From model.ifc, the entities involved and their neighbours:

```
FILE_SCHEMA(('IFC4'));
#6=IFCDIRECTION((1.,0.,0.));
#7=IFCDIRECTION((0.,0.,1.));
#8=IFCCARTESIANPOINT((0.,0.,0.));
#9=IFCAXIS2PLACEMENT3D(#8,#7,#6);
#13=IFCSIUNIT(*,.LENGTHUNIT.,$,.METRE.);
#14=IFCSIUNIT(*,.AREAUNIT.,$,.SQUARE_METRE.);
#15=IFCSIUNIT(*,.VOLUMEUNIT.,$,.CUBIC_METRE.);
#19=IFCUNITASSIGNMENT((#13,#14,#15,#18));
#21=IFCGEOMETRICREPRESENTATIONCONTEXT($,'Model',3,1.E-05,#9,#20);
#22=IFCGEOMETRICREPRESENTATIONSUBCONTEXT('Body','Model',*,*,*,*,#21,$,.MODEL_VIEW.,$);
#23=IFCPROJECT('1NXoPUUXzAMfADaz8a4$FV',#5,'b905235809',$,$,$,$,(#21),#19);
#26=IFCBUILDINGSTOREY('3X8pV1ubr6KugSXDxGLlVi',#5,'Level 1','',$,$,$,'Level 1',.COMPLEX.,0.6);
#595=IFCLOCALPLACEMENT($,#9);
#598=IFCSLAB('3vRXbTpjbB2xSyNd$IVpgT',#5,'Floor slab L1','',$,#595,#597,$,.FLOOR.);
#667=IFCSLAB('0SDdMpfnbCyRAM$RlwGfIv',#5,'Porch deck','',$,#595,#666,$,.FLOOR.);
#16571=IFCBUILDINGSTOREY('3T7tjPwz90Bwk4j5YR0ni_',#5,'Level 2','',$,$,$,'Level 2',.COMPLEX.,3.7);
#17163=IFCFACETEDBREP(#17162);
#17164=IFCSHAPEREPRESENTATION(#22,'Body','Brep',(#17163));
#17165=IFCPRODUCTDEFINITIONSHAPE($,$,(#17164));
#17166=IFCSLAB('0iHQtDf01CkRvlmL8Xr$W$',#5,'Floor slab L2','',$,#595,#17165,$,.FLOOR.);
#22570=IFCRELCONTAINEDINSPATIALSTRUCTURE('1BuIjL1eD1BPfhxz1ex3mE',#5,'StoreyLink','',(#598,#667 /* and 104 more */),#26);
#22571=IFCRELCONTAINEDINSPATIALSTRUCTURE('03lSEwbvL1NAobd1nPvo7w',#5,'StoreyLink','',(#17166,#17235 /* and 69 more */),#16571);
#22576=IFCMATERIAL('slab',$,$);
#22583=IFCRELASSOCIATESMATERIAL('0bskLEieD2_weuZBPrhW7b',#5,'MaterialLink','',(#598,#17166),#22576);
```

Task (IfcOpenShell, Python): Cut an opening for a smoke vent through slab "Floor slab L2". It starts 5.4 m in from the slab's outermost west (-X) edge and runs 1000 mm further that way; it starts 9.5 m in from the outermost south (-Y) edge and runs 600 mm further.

```python
import numpy as np
import ifcopenshell
import ifcopenshell.api.feature
import ifcopenshell.api.geometry
import ifcopenshell.api.root
import ifcopenshell.geom
import ifcopenshell.util.placement
import ifcopenshell.util.representation
import ifcopenshell.util.shape
import ifcopenshell.util.unit

model = ifcopenshell.open("model.ifc")
unit_scale = ifcopenshell.util.unit.calculate_unit_scale(model)
settings = ifcopenshell.geom.settings()


def volume(element):
    """Net volume in cubic metres, openings subtracted."""
    shape = ifcopenshell.geom.create_shape(settings, element)
    return ifcopenshell.util.shape.get_volume(shape.geometry)


slab = model.by_guid("0iHQtDf01CkRvlmL8Xr$W$")
before = volume(slab)

# Extent in the slab's own axes, in metres. The edges named are its -X and -Y sides.
slab_shape = ifcopenshell.geom.create_shape(settings, slab)
vertices = ifcopenshell.util.shape.get_vertices(slab_shape.geometry)
x_min, y_min, bottom = vertices.min(axis=0)
top = vertices[:, 2].max()

opening = ifcopenshell.api.root.create_entity(model, ifc_class="IfcOpeningElement", name="Smoke vent opening", predefined_type="OPENING")
context = ifcopenshell.util.representation.get_context(model, "Model", "Body", "MODEL_VIEW")
width, depth = 1, 0.6
outline = [(0.0, 0.0), (width, 0.0), (width, depth), (0.0, depth), (0.0, 0.0)]
# Overshoot both faces by 50 mm so the cut is clean.
shape = ifcopenshell.api.geometry.add_slab_representation(
    model, context=context, depth=top - bottom + 0.1, polyline=outline
)
ifcopenshell.api.geometry.assign_representation(model, product=opening, representation=shape)

matrix = ifcopenshell.util.placement.get_local_placement(slab.ObjectPlacement)
matrix[:, 3] = matrix @ np.append(np.array([x_min + 5.4, y_min + 9.5, bottom - 0.05]) / unit_scale, 1.0)
ifcopenshell.api.geometry.edit_object_placement(model, product=opening, matrix=matrix, is_si=False)
ifcopenshell.api.feature.add_feature(model, feature=opening, element=slab)

after = volume(slab)

print(f"slab volume {before:.3f} -> {after:.3f} m3")

model.write("model_v2.ifc")
```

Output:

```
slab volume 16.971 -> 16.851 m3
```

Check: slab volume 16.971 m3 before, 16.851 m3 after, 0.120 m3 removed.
